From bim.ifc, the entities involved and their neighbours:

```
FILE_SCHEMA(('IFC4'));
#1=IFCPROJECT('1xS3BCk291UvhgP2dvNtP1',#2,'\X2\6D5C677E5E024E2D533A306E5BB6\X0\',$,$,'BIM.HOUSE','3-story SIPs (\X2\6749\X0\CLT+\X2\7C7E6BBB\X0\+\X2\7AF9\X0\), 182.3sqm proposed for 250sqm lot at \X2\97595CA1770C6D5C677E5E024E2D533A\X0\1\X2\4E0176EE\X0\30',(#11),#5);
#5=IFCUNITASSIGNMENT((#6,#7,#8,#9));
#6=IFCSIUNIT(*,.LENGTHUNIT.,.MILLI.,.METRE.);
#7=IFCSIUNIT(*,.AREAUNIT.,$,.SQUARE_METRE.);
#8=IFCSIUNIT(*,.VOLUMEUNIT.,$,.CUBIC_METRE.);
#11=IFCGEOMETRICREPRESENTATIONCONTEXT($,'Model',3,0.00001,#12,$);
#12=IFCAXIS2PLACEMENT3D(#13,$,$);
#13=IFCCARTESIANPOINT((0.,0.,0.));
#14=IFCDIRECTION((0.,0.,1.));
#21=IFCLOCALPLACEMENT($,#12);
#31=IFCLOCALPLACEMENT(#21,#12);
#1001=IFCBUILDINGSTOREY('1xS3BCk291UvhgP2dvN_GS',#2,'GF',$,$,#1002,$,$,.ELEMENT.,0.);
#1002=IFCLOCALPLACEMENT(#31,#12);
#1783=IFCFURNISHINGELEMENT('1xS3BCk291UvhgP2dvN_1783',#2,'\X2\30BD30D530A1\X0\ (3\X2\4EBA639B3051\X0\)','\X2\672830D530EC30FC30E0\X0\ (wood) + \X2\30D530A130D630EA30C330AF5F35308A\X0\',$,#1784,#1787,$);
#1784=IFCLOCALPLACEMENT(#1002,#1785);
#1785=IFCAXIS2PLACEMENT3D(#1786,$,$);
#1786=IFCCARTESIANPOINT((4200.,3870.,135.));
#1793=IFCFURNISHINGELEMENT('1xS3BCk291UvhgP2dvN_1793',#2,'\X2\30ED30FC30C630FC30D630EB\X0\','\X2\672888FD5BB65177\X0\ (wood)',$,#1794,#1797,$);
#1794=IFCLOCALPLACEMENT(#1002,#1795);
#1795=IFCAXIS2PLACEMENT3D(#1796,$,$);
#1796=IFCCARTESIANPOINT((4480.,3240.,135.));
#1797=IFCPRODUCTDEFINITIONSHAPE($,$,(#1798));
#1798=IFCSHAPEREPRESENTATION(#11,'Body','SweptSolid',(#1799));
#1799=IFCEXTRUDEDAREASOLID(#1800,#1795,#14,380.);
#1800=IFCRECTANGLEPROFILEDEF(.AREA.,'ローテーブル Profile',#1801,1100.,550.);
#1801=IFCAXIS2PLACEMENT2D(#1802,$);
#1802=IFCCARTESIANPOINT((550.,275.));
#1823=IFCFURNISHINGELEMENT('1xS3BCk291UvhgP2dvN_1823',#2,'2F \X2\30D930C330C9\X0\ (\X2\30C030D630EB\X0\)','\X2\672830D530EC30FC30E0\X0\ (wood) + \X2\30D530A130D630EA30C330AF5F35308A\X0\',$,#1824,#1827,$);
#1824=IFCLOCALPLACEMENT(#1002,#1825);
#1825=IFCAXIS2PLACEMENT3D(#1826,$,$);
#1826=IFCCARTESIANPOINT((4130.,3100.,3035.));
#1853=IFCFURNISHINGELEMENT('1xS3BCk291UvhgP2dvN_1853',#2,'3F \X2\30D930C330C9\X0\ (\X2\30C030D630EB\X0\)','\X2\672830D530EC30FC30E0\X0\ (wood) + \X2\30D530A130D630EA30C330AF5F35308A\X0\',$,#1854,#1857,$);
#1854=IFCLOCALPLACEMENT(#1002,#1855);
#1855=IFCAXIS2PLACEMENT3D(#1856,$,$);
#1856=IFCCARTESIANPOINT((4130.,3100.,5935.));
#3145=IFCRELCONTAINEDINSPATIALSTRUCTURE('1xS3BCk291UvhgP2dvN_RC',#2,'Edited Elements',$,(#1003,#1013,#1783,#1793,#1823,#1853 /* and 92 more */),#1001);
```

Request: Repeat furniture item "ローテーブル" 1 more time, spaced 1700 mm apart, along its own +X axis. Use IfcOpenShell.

```python
import ifcopenshell
import ifcopenshell.api.geometry
import ifcopenshell.api.root
import ifcopenshell.util.element
import ifcopenshell.util.placement
import ifcopenshell.util.unit

model = ifcopenshell.open("bim.ifc")
unit_scale = ifcopenshell.util.unit.calculate_unit_scale(model)


def reuse_history(source, copy):
    """copy_class also copies each property set's owner history, people and application; keep the originals."""
    for rel in copy.IsDefinedBy:
        if rel.is_a("IfcRelDefinesByProperties") and (history := rel.RelatingPropertyDefinition.OwnerHistory):
            rel.RelatingPropertyDefinition.OwnerHistory = source.OwnerHistory
            ifcopenshell.util.element.remove_deep2(model, history)


source = model.by_guid("1xS3BCk291UvhgP2dvN_1793")
base = ifcopenshell.util.placement.get_local_placement(source.ObjectPlacement)
step = base[:3, 0] * 1.7 / unit_scale

for i in range(1, 2):
    copy = ifcopenshell.api.root.copy_class(model, product=source)
    copy.Representation = ifcopenshell.util.element.copy_deep(
        model, source.Representation, exclude=["IfcGeometricRepresentationContext", "IfcRepresentationMap"]
    )
    reuse_history(source, copy)
    matrix = base.copy()
    matrix[:3, 3] += i * step
    print("added at", matrix[:3, 3].round(3) + 0.0)
    ifcopenshell.api.geometry.edit_object_placement(model, product=copy, matrix=matrix, is_si=False)

model.write("bim-out.ifc")
```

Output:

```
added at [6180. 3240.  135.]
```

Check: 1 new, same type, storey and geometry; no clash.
